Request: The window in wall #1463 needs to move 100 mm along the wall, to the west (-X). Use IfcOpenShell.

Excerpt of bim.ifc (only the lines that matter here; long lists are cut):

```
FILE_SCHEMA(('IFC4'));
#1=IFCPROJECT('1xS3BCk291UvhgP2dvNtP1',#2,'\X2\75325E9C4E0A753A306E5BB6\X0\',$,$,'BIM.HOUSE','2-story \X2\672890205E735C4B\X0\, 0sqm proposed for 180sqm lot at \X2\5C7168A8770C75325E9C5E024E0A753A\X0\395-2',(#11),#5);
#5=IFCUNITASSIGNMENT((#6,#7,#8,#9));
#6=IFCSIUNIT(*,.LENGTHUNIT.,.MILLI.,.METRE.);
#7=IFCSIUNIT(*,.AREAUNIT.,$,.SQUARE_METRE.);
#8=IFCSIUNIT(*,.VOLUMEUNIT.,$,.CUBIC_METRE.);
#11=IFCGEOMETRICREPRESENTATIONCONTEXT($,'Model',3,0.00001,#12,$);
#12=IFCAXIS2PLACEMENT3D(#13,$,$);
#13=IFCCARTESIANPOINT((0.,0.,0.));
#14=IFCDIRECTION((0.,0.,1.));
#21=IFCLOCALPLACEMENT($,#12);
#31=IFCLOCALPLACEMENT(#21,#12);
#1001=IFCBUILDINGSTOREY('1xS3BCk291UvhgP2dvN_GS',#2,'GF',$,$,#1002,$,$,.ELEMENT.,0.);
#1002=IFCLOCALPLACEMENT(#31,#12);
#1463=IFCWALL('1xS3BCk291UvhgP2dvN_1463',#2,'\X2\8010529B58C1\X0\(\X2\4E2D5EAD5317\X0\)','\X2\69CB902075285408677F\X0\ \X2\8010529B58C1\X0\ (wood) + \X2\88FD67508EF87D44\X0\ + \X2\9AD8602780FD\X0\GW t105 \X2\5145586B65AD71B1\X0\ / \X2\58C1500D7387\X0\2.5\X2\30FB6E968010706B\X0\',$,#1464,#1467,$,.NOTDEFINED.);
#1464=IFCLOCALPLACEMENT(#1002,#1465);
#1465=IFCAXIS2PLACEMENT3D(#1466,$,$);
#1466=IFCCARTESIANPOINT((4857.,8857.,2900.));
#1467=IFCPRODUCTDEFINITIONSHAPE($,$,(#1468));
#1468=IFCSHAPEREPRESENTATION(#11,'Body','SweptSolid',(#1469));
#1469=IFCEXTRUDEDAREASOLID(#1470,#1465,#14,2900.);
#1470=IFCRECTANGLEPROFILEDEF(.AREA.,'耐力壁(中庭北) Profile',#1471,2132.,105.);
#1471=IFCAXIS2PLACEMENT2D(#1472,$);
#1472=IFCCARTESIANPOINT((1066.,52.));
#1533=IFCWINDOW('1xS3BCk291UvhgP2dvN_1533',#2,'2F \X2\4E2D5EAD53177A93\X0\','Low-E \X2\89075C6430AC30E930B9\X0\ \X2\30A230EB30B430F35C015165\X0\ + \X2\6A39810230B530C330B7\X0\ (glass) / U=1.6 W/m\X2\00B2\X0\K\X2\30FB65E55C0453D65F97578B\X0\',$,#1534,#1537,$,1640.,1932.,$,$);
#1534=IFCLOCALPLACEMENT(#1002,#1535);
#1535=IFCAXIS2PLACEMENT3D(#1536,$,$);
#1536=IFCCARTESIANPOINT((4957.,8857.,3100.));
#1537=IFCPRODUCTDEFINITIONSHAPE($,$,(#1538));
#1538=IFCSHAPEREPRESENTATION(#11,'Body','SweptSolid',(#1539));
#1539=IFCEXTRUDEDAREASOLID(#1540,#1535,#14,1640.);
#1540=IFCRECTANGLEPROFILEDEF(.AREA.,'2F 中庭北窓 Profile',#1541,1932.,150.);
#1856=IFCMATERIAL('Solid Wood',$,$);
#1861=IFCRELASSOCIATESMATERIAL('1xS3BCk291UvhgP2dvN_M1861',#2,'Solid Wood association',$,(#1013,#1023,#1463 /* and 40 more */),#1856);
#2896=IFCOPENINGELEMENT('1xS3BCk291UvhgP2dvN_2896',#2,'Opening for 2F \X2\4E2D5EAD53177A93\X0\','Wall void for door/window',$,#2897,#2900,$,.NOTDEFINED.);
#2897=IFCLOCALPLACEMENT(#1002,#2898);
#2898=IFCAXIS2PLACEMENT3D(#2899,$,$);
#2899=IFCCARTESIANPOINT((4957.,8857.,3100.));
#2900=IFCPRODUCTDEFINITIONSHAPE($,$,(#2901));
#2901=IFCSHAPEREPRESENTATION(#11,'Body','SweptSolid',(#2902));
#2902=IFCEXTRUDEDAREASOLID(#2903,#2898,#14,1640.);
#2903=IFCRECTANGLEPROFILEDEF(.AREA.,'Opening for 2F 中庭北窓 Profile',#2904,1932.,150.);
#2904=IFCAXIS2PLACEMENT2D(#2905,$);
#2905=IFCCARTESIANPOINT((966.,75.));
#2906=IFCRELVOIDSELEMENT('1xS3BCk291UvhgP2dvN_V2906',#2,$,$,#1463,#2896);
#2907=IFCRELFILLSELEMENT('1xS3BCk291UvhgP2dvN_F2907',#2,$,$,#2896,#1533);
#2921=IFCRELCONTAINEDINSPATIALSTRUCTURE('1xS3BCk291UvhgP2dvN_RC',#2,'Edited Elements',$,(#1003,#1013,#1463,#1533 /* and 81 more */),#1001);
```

```python
import ifcopenshell
import ifcopenshell.api.geometry
import ifcopenshell.util.placement
import ifcopenshell.util.unit

model = ifcopenshell.open("bim.ifc")
unit_scale = ifcopenshell.util.unit.calculate_unit_scale(model)

window = model.by_id(1533)
opening = window.FillsVoids[0].RelatingOpeningElement
wall = opening.VoidsElements[0].RelatingBuildingElement

wall_matrix = ifcopenshell.util.placement.get_local_placement(wall.ObjectPlacement)
shift = wall_matrix[:3, 0] * -0.1 / unit_scale
before = ifcopenshell.util.placement.get_local_placement(window.ObjectPlacement)[:3, 3].copy()

# The window is not placed relative to its opening, so move both.
for product in (opening, window):
    matrix = ifcopenshell.util.placement.get_local_placement(product.ObjectPlacement)
    matrix[:3, 3] += shift
    ifcopenshell.api.geometry.edit_object_placement(model, product=product, matrix=matrix, is_si=False)

after = ifcopenshell.util.placement.get_local_placement(window.ObjectPlacement)[:3, 3]
print("window moved by", (after - before).round(3) + 0.0)

model.write("bim_rev.ifc")
```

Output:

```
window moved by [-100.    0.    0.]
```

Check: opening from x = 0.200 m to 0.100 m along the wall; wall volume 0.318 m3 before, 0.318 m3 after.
